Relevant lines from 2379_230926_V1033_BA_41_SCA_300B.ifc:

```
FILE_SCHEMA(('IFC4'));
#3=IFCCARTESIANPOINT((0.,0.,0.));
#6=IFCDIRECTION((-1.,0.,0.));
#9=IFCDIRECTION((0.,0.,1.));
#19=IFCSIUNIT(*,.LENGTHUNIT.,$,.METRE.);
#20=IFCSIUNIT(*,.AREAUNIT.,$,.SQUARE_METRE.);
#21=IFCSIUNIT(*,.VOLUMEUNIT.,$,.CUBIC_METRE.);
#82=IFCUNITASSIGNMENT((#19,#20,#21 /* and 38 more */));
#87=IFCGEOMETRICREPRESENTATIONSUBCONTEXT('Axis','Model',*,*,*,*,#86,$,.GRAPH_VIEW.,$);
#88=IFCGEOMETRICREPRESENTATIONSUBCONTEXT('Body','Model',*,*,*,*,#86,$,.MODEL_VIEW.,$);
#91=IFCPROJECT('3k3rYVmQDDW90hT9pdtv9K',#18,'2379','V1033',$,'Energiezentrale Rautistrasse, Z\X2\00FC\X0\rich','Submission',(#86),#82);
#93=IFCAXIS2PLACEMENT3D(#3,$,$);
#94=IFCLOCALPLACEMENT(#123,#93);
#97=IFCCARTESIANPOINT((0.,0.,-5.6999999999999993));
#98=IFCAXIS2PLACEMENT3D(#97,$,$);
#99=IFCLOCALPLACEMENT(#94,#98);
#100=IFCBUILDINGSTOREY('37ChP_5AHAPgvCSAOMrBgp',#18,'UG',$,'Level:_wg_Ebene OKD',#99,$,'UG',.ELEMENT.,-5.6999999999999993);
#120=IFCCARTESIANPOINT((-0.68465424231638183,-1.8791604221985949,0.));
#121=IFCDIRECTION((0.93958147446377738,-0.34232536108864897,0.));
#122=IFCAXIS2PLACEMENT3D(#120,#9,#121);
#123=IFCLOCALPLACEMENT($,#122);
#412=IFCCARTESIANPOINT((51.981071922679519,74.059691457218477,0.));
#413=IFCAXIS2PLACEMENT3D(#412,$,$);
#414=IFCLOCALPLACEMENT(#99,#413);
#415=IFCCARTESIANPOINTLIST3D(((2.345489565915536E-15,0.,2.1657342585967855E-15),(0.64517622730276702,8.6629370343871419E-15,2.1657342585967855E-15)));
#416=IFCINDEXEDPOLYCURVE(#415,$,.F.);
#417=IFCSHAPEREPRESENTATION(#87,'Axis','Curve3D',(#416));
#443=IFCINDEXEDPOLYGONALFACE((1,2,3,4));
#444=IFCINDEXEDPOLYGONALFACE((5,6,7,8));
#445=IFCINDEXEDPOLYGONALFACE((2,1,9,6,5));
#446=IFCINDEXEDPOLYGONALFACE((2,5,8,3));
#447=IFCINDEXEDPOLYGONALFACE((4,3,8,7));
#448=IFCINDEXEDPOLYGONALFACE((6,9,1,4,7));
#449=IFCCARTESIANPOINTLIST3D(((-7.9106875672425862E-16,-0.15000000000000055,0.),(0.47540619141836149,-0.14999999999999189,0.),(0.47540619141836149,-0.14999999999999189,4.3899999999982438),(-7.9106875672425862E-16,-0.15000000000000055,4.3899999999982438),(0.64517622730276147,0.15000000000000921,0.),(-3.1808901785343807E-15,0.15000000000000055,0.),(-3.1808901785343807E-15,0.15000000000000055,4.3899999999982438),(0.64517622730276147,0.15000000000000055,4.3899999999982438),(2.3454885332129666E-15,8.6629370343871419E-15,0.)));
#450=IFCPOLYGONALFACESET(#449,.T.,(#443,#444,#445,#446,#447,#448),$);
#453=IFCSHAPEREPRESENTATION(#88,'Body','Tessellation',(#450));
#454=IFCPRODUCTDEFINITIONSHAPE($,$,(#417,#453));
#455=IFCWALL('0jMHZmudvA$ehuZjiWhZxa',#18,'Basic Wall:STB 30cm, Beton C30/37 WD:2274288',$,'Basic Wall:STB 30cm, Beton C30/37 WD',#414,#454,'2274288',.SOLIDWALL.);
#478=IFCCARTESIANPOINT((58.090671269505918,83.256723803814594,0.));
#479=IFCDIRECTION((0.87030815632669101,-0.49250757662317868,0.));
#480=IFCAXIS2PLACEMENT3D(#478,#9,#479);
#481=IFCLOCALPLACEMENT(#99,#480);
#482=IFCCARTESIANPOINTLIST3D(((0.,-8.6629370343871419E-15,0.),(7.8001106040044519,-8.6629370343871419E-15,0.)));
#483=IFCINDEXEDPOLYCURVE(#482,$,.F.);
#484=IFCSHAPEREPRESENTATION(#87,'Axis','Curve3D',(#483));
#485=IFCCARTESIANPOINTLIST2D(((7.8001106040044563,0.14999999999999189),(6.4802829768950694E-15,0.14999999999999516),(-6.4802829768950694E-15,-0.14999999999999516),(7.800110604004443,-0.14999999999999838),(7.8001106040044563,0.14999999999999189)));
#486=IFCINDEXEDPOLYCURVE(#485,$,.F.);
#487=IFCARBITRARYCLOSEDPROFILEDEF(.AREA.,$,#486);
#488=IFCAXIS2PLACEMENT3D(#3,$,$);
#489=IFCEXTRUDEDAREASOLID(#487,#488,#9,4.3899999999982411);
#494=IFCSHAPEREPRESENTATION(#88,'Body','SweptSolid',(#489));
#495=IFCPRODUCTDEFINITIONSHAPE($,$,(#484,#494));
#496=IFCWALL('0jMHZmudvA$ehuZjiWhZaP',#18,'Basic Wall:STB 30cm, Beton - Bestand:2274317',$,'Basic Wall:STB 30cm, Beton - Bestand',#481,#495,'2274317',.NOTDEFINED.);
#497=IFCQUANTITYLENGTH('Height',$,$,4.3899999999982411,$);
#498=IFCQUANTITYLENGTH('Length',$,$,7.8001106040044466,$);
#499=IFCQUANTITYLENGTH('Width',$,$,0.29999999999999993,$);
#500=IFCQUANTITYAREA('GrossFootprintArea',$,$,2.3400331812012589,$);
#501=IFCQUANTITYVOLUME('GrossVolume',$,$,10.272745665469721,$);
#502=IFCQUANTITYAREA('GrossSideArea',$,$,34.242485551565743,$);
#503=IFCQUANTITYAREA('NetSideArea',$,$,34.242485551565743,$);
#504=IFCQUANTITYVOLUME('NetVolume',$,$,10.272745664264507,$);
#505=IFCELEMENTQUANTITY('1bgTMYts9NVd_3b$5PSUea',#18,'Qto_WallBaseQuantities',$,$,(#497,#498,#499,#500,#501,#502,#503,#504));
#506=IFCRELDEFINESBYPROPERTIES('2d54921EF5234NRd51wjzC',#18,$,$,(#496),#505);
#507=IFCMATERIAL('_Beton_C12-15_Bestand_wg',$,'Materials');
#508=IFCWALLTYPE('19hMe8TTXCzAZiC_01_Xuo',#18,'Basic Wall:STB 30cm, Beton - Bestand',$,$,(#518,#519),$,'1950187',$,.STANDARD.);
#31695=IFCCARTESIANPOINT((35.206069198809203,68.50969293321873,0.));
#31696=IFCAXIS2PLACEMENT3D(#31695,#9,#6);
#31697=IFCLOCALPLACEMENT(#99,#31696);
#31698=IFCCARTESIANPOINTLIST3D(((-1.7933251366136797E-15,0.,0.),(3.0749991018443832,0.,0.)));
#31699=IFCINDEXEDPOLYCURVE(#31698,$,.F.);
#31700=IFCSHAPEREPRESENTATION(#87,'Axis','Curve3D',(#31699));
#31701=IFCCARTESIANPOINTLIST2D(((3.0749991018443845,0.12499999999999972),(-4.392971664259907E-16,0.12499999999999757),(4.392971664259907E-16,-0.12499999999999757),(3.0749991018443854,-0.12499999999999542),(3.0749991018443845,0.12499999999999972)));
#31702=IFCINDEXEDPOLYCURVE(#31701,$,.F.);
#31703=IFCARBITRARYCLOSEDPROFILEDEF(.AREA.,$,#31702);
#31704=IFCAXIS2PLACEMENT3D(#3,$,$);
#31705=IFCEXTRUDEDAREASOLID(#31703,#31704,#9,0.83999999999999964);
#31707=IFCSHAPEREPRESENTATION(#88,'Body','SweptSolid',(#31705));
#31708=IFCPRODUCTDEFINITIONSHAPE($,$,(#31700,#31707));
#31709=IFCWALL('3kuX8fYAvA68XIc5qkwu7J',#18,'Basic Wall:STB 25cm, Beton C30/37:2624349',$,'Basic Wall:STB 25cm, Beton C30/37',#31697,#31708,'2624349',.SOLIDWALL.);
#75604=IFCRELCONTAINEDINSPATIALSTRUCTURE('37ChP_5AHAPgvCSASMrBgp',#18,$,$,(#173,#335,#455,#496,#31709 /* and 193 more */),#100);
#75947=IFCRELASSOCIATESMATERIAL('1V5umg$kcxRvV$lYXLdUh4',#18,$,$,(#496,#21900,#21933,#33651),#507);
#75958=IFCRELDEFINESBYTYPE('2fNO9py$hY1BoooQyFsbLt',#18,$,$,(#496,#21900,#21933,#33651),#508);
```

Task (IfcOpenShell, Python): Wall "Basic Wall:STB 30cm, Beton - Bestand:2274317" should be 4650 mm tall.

```python
import ifcopenshell
import ifcopenshell.api.pset
import ifcopenshell.geom
import ifcopenshell.util.element
import ifcopenshell.util.representation
import ifcopenshell.util.shape
import ifcopenshell.util.unit

model = ifcopenshell.open("2379_230926_V1033_BA_41_SCA_300B.ifc")
unit_scale = ifcopenshell.util.unit.calculate_unit_scale(model)
area_scale = ifcopenshell.util.unit.calculate_unit_scale(model, "AREAUNIT")
volume_scale = ifcopenshell.util.unit.calculate_unit_scale(model, "VOLUMEUNIT")
settings = ifcopenshell.geom.settings()


def volume(element):
    """Net volume in cubic metres, openings subtracted."""
    shape = ifcopenshell.geom.create_shape(settings, element)
    return ifcopenshell.util.shape.get_volume(shape.geometry)


wall = model.by_id(496)
before = volume(wall)

body = ifcopenshell.util.representation.get_representation(wall, "Model", "Body")
solid = body.Items[0]
old_height = solid.Depth
solid.Depth = 4.65 / unit_scale
after = volume(wall)
thickness = 0.3  # wall thickness in metres

# Update the stored height, areas and volumes.
qto = model.by_id(ifcopenshell.util.element.get_pset(wall, "Qto_WallBaseQuantities", should_inherit=False)["id"])
ifcopenshell.api.pset.edit_qto(model, qto=qto, properties={
    "Height": solid.Depth,
    "GrossVolume": ifcopenshell.util.element.get_pset(wall, "Qto_WallBaseQuantities", "GrossVolume") * solid.Depth / old_height,
    "GrossSideArea": ifcopenshell.util.element.get_pset(wall, "Qto_WallBaseQuantities", "GrossSideArea") * solid.Depth / old_height,
    "NetSideArea": after / thickness / area_scale,
    "NetVolume": after / volume_scale,
})

print(f"height {old_height:g} -> {solid.Depth:g}, volume {before:.3f} -> {after:.3f} m3")

model.write("2379_230926_V1033_BA_41_SCA_300B_v2.ifc")
```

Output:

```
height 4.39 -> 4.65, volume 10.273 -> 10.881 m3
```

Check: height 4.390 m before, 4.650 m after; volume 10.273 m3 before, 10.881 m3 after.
